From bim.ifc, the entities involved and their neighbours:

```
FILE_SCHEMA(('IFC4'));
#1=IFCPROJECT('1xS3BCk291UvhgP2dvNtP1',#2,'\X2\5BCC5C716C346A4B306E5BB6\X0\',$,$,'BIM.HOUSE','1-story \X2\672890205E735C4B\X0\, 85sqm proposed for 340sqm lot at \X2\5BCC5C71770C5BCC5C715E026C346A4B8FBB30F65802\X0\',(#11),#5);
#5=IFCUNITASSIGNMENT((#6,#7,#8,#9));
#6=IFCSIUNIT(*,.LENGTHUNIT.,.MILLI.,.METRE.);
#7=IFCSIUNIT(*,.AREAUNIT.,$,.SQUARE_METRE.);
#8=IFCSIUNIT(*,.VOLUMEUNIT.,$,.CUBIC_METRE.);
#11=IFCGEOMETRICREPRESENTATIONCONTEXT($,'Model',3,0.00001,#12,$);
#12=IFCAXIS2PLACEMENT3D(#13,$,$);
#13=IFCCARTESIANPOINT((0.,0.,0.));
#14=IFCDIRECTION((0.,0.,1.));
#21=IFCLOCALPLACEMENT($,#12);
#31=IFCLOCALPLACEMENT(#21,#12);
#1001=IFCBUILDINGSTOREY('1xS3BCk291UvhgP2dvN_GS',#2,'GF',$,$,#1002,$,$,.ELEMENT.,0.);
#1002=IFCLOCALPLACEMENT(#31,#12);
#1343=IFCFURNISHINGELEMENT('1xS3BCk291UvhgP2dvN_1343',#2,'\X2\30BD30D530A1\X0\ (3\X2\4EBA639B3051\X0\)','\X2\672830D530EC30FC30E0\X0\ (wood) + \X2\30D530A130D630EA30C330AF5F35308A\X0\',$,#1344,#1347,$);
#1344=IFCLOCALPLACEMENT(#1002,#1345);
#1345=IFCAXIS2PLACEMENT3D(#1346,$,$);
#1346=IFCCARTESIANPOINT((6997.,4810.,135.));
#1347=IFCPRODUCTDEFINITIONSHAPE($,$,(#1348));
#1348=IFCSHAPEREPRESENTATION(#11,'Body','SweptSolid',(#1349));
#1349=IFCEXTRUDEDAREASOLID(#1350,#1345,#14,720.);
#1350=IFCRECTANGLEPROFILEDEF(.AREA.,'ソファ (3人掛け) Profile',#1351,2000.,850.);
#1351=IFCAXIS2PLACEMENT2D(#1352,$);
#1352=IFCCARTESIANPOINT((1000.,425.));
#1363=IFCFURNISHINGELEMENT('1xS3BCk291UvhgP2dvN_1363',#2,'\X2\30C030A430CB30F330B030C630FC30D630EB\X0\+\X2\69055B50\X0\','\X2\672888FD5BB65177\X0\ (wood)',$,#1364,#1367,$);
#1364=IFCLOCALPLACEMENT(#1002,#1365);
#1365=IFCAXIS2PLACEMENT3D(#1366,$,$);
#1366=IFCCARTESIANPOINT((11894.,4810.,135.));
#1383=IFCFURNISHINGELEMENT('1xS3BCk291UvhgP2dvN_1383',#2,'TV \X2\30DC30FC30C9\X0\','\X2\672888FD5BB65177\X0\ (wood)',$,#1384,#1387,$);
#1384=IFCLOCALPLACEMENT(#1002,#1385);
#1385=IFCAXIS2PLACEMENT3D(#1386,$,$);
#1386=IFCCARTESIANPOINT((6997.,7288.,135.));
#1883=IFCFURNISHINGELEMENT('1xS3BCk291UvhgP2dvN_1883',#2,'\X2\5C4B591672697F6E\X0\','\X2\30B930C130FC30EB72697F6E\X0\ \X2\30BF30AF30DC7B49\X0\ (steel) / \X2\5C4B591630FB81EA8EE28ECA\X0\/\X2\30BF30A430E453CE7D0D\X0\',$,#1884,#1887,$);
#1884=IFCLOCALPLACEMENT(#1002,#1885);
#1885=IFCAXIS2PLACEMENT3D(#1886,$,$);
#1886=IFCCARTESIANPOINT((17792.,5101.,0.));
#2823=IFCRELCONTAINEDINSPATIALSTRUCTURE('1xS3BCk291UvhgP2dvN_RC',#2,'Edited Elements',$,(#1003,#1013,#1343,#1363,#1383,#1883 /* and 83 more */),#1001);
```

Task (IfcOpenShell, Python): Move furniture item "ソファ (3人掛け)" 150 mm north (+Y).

```python
import ifcopenshell
import ifcopenshell.api.geometry
import ifcopenshell.util.placement
import ifcopenshell.util.unit

model = ifcopenshell.open("bim.ifc")
unit_scale = ifcopenshell.util.unit.calculate_unit_scale(model)

item = model.by_id(1343)
matrix = ifcopenshell.util.placement.get_local_placement(item.ObjectPlacement)
matrix[1, 3] += 0.15 / unit_scale
ifcopenshell.api.geometry.edit_object_placement(model, product=item, matrix=matrix, is_si=False)

print(ifcopenshell.util.placement.get_local_placement(item.ObjectPlacement).round(3) + 0.0)

model.write("bim_v2.ifc")
```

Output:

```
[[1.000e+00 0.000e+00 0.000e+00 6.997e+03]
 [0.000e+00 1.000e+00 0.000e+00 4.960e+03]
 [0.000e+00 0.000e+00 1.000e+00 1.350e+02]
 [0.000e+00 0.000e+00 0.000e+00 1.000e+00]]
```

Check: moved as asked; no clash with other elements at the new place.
